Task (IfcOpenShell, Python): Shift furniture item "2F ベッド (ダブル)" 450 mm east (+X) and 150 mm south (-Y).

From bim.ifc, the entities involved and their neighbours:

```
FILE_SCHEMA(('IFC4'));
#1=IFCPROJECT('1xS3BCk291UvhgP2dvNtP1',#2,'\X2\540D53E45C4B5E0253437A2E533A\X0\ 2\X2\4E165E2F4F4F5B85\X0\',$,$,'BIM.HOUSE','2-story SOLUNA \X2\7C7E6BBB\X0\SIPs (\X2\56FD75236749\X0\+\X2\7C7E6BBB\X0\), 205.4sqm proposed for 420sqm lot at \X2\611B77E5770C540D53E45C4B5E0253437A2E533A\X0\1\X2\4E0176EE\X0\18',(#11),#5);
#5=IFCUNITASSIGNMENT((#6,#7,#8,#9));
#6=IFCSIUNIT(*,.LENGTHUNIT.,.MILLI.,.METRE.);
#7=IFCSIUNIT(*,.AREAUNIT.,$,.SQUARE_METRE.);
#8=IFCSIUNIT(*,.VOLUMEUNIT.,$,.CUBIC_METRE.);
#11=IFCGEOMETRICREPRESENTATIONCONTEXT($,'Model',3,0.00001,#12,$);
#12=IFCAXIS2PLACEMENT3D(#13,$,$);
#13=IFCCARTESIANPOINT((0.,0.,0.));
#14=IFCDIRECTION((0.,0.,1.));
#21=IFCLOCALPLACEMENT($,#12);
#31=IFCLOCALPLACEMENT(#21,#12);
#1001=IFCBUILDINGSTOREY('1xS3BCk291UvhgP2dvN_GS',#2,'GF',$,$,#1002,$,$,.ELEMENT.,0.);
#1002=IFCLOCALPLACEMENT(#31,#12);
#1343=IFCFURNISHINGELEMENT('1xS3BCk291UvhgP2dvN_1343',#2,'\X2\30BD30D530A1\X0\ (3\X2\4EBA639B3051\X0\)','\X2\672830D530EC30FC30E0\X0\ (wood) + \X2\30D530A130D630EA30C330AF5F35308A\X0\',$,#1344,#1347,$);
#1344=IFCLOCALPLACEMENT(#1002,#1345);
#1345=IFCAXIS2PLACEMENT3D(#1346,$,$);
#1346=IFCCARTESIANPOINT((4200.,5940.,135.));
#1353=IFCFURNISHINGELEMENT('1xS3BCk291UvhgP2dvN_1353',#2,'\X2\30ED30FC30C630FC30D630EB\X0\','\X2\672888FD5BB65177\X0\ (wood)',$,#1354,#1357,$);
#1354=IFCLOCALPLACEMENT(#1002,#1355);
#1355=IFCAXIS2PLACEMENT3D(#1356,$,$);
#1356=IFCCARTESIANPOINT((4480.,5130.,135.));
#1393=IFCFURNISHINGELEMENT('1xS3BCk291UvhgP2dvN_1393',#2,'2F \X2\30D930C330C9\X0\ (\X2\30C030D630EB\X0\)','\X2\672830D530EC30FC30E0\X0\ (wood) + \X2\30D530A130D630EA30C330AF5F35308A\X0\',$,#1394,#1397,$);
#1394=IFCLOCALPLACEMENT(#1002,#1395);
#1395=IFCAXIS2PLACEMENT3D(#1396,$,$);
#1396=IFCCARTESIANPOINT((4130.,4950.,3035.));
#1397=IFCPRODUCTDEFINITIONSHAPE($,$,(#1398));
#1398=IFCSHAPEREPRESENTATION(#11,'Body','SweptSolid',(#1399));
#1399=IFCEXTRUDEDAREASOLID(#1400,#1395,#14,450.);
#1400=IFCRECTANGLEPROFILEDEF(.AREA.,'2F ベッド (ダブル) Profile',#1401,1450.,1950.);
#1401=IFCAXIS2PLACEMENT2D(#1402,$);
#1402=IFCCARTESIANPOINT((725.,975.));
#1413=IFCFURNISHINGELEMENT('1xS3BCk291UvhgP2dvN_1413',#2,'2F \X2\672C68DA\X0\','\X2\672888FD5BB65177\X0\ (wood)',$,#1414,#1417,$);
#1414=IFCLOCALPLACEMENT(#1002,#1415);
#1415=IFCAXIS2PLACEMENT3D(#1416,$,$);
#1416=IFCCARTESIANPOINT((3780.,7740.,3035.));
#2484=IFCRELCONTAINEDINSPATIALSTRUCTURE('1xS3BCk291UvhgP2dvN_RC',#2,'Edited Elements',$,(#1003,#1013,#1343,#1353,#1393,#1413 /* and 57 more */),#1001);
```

```python
import ifcopenshell
import ifcopenshell.api.geometry
import ifcopenshell.util.placement
import ifcopenshell.util.unit

model = ifcopenshell.open("bim.ifc")
unit_scale = ifcopenshell.util.unit.calculate_unit_scale(model)

item = model.by_id(1393)
matrix = ifcopenshell.util.placement.get_local_placement(item.ObjectPlacement)
matrix[0, 3] += 0.45 / unit_scale
matrix[1, 3] -= 0.15 / unit_scale
ifcopenshell.api.geometry.edit_object_placement(model, product=item, matrix=matrix, is_si=False)

print(ifcopenshell.util.placement.get_local_placement(item.ObjectPlacement).round(3) + 0.0)

model.write("bim_updated.ifc")
```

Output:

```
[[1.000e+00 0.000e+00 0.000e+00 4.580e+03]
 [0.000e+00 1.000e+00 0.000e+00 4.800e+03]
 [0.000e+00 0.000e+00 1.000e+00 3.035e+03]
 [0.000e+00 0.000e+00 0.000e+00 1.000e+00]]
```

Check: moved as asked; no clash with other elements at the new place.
